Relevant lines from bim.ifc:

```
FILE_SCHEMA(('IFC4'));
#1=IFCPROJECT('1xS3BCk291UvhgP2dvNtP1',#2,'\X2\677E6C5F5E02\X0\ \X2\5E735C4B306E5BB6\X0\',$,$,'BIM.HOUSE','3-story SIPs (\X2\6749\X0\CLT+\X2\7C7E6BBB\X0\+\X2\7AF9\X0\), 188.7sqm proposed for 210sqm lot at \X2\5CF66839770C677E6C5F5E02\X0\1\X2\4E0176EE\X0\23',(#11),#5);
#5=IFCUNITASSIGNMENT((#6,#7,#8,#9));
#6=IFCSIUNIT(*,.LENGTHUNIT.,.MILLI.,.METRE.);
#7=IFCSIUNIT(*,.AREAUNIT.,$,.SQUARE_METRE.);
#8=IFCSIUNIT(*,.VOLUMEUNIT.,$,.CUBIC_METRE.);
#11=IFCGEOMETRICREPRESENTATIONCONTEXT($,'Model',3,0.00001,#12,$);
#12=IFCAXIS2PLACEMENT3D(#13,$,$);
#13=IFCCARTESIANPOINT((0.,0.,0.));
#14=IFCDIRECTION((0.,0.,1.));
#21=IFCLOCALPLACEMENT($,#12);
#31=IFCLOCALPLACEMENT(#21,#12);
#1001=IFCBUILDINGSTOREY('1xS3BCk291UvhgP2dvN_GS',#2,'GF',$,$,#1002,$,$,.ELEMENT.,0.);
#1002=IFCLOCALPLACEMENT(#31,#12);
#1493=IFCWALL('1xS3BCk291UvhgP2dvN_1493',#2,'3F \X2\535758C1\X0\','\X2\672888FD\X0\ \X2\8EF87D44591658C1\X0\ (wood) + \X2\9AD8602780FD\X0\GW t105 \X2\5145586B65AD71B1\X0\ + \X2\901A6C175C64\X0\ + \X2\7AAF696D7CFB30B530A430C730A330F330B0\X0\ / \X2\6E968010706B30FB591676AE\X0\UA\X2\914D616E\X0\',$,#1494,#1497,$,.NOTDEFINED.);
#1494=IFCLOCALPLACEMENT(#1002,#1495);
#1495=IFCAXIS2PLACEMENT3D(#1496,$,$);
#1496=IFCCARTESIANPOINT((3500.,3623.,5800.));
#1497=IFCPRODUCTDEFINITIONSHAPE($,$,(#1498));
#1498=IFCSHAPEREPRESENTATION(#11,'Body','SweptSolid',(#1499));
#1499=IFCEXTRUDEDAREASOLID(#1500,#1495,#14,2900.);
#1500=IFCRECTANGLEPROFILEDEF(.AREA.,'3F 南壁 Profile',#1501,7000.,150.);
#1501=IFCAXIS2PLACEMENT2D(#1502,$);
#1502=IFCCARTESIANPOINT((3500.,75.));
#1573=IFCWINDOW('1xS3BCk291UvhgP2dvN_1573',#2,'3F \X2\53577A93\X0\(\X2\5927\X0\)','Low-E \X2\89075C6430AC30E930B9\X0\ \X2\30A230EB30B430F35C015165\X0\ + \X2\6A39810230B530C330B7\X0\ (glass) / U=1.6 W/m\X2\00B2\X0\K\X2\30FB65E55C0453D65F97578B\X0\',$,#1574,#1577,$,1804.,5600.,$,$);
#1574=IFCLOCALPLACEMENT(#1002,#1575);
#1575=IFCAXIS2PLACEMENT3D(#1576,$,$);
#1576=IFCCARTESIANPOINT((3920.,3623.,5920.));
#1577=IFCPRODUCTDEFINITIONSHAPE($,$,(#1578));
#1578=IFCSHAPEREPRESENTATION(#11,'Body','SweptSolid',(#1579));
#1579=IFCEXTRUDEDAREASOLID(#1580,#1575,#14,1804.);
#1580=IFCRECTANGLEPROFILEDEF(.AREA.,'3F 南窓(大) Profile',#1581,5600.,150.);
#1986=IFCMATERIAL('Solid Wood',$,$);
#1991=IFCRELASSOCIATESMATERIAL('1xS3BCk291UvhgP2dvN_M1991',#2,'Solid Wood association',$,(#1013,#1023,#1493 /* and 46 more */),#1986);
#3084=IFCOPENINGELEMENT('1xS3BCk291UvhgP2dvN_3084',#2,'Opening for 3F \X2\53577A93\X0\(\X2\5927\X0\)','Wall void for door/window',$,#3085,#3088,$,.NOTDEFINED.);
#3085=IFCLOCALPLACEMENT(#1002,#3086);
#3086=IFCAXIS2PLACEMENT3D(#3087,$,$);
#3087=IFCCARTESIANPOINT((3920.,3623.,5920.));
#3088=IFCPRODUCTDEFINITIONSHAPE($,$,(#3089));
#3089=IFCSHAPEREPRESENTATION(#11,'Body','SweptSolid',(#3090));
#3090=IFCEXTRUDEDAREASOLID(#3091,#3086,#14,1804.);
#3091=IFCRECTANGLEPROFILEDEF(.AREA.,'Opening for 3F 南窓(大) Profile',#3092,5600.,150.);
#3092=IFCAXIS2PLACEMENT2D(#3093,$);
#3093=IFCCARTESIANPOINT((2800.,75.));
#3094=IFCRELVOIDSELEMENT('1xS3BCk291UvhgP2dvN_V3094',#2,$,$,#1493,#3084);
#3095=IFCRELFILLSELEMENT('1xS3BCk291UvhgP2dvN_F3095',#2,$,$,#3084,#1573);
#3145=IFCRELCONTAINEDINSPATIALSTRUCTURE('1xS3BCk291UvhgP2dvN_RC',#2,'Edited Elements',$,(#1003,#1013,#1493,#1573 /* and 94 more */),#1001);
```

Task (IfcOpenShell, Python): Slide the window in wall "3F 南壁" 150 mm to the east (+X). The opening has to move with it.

```python
import ifcopenshell
import ifcopenshell.api.geometry
import ifcopenshell.util.placement
import ifcopenshell.util.unit

model = ifcopenshell.open("bim.ifc")
unit_scale = ifcopenshell.util.unit.calculate_unit_scale(model)

window = model.by_guid("1xS3BCk291UvhgP2dvN_1573")
opening = window.FillsVoids[0].RelatingOpeningElement
wall = opening.VoidsElements[0].RelatingBuildingElement

wall_matrix = ifcopenshell.util.placement.get_local_placement(wall.ObjectPlacement)
shift = wall_matrix[:3, 0] * 0.15 / unit_scale
before = ifcopenshell.util.placement.get_local_placement(window.ObjectPlacement)[:3, 3].copy()

# The window is not placed relative to its opening, so move both.
for product in (opening, window):
    matrix = ifcopenshell.util.placement.get_local_placement(product.ObjectPlacement)
    matrix[:3, 3] += shift
    ifcopenshell.api.geometry.edit_object_placement(model, product=product, matrix=matrix, is_si=False)

after = ifcopenshell.util.placement.get_local_placement(window.ObjectPlacement)[:3, 3]
print("window moved by", (after - before).round(3) + 0.0)

model.write("bim_updated.ifc")
```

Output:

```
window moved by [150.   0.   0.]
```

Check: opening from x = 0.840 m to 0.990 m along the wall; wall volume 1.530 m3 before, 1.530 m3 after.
